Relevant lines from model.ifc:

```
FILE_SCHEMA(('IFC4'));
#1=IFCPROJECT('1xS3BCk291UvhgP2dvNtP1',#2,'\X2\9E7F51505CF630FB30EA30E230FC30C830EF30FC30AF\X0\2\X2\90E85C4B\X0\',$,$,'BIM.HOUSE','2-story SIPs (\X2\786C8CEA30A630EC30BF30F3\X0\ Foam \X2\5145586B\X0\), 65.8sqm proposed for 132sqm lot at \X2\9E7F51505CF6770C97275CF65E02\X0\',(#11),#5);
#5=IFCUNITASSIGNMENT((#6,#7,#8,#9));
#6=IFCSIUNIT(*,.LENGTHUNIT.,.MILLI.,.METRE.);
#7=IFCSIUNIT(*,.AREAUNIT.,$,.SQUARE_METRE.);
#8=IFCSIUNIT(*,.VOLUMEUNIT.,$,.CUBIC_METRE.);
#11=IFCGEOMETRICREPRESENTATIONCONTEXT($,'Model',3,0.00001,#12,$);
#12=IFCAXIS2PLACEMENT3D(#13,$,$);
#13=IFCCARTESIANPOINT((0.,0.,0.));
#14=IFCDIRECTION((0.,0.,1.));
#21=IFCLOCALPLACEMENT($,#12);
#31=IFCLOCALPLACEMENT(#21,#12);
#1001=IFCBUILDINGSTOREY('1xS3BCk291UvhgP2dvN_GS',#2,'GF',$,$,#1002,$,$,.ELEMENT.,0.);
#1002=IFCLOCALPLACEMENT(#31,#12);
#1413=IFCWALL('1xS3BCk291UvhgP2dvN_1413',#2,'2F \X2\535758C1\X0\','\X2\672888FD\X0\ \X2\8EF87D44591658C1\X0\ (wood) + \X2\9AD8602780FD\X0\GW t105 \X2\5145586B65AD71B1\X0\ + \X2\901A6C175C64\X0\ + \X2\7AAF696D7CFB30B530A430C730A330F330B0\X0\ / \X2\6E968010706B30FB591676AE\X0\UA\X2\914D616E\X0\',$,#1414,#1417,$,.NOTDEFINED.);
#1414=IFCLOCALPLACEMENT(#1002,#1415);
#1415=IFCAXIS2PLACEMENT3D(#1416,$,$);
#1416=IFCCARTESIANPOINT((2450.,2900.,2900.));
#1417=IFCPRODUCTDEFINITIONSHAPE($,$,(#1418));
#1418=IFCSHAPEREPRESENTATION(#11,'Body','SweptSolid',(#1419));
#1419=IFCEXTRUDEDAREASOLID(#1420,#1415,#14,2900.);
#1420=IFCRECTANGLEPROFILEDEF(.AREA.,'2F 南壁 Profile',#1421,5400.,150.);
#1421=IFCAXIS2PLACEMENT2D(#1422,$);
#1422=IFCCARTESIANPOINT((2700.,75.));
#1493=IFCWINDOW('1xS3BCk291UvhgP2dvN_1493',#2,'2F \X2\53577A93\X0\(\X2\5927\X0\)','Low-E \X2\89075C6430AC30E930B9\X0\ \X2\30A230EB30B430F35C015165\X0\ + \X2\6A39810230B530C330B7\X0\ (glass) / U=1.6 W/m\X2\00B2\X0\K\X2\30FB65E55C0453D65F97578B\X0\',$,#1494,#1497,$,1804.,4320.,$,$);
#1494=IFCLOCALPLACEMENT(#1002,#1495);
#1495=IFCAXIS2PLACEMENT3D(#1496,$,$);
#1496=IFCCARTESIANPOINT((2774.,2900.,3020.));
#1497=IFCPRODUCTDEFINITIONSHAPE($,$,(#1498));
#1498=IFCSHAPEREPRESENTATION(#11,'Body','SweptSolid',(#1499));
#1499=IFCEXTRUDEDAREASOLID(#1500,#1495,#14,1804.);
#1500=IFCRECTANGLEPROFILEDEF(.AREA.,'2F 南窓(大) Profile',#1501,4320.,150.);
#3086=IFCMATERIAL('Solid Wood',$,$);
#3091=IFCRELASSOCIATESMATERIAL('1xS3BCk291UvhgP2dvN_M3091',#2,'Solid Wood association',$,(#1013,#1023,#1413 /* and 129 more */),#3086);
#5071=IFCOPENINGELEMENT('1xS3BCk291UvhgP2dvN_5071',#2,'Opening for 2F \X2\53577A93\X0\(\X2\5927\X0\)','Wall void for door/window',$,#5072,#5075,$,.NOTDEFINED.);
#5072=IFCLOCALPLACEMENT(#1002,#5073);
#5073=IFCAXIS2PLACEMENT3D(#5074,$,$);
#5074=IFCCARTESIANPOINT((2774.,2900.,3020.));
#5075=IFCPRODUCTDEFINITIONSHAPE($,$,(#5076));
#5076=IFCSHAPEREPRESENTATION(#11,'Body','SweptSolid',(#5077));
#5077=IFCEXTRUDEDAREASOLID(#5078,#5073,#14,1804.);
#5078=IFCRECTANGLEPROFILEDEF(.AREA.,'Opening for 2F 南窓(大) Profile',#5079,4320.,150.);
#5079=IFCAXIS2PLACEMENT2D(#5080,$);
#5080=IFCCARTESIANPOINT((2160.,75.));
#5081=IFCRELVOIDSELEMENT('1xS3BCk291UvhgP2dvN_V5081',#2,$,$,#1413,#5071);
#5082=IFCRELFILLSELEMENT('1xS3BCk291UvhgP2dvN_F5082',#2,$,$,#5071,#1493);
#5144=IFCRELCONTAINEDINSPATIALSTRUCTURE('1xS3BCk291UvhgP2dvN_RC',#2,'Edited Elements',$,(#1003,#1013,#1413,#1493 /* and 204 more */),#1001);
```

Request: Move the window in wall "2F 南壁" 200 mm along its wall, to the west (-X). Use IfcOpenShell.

```python
import ifcopenshell
import ifcopenshell.api.geometry
import ifcopenshell.util.placement
import ifcopenshell.util.unit

model = ifcopenshell.open("model.ifc")
unit_scale = ifcopenshell.util.unit.calculate_unit_scale(model)

window = model.by_id(1493)
opening = window.FillsVoids[0].RelatingOpeningElement
wall = opening.VoidsElements[0].RelatingBuildingElement

wall_matrix = ifcopenshell.util.placement.get_local_placement(wall.ObjectPlacement)
shift = wall_matrix[:3, 0] * -0.2 / unit_scale
before = ifcopenshell.util.placement.get_local_placement(window.ObjectPlacement)[:3, 3].copy()

# The window is not placed relative to its opening, so move both.
for product in (opening, window):
    matrix = ifcopenshell.util.placement.get_local_placement(product.ObjectPlacement)
    matrix[:3, 3] += shift
    ifcopenshell.api.geometry.edit_object_placement(model, product=product, matrix=matrix, is_si=False)

after = ifcopenshell.util.placement.get_local_placement(window.ObjectPlacement)[:3, 3]
print("window moved by", (after - before).round(3) + 0.0)

model.write("model_rev.ifc")
```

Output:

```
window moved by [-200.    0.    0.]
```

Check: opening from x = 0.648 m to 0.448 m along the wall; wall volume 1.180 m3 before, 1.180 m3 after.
